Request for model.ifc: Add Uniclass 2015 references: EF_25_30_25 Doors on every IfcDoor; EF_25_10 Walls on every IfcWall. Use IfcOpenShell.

First a look at what the model holds.

```python
import ifcopenshell

model = ifcopenshell.open("model.ifc")
print(model.schema)
print("classifications:", [c.Name for c in model.by_type("IfcClassification")])
for ifc_class in ("IfcDoor", "IfcRoof", "IfcStair", "IfcWall", "IfcWindow"):
    print(ifc_class, len(model.by_type(ifc_class)))
```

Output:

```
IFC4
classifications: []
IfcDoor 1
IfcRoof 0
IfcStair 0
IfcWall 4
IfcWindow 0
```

```python
import ifcopenshell
import ifcopenshell.api.classification

model = ifcopenshell.open("model.ifc")

system = ifcopenshell.api.classification.add_classification(model, classification="Uniclass 2015")

codes = {
    "IfcDoor": ("EF_25_30_25", "Doors"),
    "IfcWall": ("EF_25_10", "Walls"),
}
for ifc_class, (code, name) in codes.items():
    products = model.by_type(ifc_class)
    ifcopenshell.api.classification.add_reference(
        model, products=products, classification=system, identification=code, name=name
    )
    print(code, len(products))

model.write("model_updated.ifc")
```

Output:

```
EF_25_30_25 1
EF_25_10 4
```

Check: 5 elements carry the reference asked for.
